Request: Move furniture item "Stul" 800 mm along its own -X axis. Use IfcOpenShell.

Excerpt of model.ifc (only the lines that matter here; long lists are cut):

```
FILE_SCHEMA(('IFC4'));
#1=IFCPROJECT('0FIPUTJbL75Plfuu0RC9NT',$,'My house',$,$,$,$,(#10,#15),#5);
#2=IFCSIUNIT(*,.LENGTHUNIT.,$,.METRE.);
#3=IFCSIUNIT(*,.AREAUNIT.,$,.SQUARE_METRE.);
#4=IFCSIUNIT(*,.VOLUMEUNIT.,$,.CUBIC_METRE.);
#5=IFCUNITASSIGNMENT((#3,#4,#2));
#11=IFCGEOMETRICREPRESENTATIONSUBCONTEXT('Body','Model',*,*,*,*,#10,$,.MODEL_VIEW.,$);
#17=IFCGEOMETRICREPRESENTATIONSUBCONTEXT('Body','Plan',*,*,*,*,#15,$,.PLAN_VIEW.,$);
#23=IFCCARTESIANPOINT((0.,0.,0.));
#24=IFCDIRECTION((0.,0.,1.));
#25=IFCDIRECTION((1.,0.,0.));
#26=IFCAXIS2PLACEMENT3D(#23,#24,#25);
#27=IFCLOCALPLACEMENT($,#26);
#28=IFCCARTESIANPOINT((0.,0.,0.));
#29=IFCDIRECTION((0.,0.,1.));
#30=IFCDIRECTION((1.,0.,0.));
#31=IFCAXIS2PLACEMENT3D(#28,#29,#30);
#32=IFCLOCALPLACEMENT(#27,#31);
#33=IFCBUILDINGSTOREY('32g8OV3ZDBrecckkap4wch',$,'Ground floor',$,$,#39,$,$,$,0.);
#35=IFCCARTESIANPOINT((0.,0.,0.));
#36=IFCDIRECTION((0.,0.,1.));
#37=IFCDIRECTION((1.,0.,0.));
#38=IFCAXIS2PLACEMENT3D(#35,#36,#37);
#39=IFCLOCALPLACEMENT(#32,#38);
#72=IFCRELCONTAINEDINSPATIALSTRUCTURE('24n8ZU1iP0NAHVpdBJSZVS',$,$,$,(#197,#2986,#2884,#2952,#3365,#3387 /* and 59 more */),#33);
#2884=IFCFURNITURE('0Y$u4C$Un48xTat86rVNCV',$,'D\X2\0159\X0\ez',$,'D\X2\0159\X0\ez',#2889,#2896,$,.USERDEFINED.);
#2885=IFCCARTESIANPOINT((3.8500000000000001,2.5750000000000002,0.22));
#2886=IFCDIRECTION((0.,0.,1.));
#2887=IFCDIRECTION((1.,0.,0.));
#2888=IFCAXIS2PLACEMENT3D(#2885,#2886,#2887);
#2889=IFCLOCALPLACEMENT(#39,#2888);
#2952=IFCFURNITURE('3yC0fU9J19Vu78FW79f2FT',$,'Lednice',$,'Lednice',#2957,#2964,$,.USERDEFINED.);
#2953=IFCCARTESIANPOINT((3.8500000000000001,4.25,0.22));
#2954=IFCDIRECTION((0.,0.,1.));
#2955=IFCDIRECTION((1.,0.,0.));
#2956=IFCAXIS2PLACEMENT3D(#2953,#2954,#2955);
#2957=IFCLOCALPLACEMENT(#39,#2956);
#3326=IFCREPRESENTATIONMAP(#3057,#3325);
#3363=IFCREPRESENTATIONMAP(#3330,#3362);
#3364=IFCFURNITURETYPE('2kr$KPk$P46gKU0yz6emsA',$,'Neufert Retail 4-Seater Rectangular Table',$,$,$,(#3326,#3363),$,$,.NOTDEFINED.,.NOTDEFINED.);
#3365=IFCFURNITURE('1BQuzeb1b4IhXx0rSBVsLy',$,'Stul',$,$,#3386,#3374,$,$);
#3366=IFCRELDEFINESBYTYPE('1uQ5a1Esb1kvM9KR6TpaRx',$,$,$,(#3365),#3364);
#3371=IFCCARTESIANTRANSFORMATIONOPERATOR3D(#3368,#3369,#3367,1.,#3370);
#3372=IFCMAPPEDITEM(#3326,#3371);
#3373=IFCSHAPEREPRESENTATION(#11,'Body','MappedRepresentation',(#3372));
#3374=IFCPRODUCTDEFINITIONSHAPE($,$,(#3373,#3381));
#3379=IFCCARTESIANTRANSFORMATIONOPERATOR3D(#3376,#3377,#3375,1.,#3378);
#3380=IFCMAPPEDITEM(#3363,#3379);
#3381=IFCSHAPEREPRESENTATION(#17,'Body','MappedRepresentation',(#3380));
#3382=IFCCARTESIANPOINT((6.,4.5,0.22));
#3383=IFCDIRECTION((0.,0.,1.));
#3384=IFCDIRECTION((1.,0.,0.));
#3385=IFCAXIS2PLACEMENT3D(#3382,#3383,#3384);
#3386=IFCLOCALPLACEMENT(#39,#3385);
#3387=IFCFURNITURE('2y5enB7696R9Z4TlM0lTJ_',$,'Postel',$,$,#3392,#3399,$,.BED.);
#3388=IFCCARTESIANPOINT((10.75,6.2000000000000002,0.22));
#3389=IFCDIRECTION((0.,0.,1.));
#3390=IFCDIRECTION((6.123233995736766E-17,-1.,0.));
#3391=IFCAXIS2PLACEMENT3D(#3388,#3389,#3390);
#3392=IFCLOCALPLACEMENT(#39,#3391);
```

```python
import ifcopenshell
import ifcopenshell.api.geometry
import ifcopenshell.util.placement
import ifcopenshell.util.unit

model = ifcopenshell.open("model.ifc")
unit_scale = ifcopenshell.util.unit.calculate_unit_scale(model)

item = model.by_id(3365)
matrix = ifcopenshell.util.placement.get_local_placement(item.ObjectPlacement)
matrix[:3, 3] -= matrix[:3, 0] * 0.8 / unit_scale
ifcopenshell.api.geometry.edit_object_placement(model, product=item, matrix=matrix, is_si=False)

print(ifcopenshell.util.placement.get_local_placement(item.ObjectPlacement).round(3) + 0.0)

model.write("model_rev.ifc")
```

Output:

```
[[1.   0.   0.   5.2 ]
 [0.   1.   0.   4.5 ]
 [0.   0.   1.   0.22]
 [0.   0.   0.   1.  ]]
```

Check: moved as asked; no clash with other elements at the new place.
